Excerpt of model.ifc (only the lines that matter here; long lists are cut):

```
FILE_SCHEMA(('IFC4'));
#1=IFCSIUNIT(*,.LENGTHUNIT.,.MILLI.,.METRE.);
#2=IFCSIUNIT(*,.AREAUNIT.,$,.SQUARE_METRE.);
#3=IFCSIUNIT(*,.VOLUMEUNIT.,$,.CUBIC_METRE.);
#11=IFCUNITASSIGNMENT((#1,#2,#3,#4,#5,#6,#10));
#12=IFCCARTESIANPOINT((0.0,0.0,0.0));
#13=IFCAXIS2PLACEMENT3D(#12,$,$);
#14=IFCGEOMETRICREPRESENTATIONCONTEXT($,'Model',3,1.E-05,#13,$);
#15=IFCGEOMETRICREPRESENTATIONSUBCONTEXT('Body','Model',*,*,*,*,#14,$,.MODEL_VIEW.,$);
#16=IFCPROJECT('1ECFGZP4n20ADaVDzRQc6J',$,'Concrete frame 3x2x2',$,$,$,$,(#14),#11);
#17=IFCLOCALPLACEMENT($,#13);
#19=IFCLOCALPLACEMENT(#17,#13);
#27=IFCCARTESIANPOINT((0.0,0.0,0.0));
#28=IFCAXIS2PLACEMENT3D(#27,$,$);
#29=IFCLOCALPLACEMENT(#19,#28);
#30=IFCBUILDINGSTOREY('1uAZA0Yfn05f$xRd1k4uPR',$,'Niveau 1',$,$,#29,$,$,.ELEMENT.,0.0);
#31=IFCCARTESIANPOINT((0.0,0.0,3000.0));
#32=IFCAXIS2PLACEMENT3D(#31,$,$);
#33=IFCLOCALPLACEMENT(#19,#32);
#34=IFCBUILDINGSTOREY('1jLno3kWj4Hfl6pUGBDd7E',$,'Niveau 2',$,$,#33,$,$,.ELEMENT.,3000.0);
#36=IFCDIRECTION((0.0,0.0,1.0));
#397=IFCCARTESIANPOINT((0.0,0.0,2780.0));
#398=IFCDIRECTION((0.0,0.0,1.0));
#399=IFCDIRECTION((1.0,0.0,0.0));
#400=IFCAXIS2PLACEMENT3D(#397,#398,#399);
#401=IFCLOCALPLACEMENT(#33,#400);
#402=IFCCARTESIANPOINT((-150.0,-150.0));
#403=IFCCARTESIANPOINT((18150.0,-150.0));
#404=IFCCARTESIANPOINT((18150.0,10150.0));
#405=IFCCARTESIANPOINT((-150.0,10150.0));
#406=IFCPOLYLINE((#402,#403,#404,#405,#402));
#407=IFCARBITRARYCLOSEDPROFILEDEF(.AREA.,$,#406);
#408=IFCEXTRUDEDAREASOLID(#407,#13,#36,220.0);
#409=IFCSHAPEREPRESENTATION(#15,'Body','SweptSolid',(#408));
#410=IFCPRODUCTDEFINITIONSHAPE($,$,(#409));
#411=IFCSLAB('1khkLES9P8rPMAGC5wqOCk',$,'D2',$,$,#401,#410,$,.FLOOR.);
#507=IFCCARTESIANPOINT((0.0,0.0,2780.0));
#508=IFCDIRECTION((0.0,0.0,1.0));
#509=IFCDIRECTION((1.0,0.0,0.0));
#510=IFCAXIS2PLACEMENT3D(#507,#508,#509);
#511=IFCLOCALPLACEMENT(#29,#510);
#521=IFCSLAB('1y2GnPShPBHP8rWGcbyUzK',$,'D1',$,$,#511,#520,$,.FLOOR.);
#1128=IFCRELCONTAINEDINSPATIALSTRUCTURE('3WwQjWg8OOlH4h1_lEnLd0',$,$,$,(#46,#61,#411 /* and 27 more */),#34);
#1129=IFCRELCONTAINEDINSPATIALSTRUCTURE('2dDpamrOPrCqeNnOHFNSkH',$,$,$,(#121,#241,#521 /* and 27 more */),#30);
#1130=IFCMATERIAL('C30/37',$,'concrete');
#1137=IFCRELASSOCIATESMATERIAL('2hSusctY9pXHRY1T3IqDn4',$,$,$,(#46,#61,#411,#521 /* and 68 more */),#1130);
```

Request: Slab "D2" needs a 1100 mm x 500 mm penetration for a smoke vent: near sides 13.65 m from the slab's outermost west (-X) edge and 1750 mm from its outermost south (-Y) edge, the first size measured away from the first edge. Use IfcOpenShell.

```python
import numpy as np
import ifcopenshell
import ifcopenshell.api.feature
import ifcopenshell.api.geometry
import ifcopenshell.api.root
import ifcopenshell.geom
import ifcopenshell.util.placement
import ifcopenshell.util.representation
import ifcopenshell.util.shape
import ifcopenshell.util.unit

model = ifcopenshell.open("model.ifc")
unit_scale = ifcopenshell.util.unit.calculate_unit_scale(model)
settings = ifcopenshell.geom.settings()


def volume(element):
    """Net volume in cubic metres, openings subtracted."""
    shape = ifcopenshell.geom.create_shape(settings, element)
    return ifcopenshell.util.shape.get_volume(shape.geometry)


slab = model.by_guid("1khkLES9P8rPMAGC5wqOCk")
before = volume(slab)

# Extent in the slab's own axes, in metres. The edges named are its -X and -Y sides.
slab_shape = ifcopenshell.geom.create_shape(settings, slab)
vertices = ifcopenshell.util.shape.get_vertices(slab_shape.geometry)
x_min, y_min, bottom = vertices.min(axis=0)
top = vertices[:, 2].max()

opening = ifcopenshell.api.root.create_entity(model, ifc_class="IfcOpeningElement", name="Smoke vent opening", predefined_type="OPENING")
context = ifcopenshell.util.representation.get_context(model, "Model", "Body", "MODEL_VIEW")
width, depth = 1.1, 0.5
outline = [(0.0, 0.0), (width, 0.0), (width, depth), (0.0, depth), (0.0, 0.0)]
# Overshoot both faces by 50 mm so the cut is clean.
shape = ifcopenshell.api.geometry.add_slab_representation(
    model, context=context, depth=top - bottom + 0.1, polyline=outline
)
ifcopenshell.api.geometry.assign_representation(model, product=opening, representation=shape)

matrix = ifcopenshell.util.placement.get_local_placement(slab.ObjectPlacement)
matrix[:, 3] = matrix @ np.append(np.array([x_min + 13.65, y_min + 1.75, bottom - 0.05]) / unit_scale, 1.0)
ifcopenshell.api.geometry.edit_object_placement(model, product=opening, matrix=matrix, is_si=False)
ifcopenshell.api.feature.add_feature(model, feature=opening, element=slab)

after = volume(slab)

print(f"slab volume {before:.3f} -> {after:.3f} m3")

model.write("model-out.ifc")
```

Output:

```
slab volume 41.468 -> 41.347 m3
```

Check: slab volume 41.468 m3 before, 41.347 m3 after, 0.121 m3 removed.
